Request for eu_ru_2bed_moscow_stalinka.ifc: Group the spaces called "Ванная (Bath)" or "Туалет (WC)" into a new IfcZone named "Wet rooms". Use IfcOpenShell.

First a look at what the model holds.

```python
import ifcopenshell

model = ifcopenshell.open("eu_ru_2bed_moscow_stalinka.ifc")
print(model.schema)
seen = {}
for space in model.by_type("IfcSpace"):
    seen[space.LongName] = seen.get(space.LongName, 0) + 1
for name, count in sorted(seen.items(), key=str):
    print(count, "x", name)
print("zones:", [z.Name for z in model.by_type("IfcZone")][:20])
```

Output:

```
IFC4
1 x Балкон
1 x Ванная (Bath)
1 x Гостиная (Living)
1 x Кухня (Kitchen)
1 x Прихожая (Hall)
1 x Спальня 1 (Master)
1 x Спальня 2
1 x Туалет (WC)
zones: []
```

```python
import ifcopenshell
import ifcopenshell.api.group
import ifcopenshell.api.root

model = ifcopenshell.open("eu_ru_2bed_moscow_stalinka.ifc")

names = {"Ванная (Bath)", "Туалет (WC)"}
spaces = [s for s in model.by_type("IfcSpace") if s.LongName in names]

zone = ifcopenshell.api.root.create_entity(model, ifc_class="IfcZone", name="Wet rooms")
ifcopenshell.api.group.assign_group(model, products=spaces, group=zone)
print(len(spaces), "spaces in", zone.Name)

model.write("eu_ru_2bed_moscow_stalinka_updated.ifc")
```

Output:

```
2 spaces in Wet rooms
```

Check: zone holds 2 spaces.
